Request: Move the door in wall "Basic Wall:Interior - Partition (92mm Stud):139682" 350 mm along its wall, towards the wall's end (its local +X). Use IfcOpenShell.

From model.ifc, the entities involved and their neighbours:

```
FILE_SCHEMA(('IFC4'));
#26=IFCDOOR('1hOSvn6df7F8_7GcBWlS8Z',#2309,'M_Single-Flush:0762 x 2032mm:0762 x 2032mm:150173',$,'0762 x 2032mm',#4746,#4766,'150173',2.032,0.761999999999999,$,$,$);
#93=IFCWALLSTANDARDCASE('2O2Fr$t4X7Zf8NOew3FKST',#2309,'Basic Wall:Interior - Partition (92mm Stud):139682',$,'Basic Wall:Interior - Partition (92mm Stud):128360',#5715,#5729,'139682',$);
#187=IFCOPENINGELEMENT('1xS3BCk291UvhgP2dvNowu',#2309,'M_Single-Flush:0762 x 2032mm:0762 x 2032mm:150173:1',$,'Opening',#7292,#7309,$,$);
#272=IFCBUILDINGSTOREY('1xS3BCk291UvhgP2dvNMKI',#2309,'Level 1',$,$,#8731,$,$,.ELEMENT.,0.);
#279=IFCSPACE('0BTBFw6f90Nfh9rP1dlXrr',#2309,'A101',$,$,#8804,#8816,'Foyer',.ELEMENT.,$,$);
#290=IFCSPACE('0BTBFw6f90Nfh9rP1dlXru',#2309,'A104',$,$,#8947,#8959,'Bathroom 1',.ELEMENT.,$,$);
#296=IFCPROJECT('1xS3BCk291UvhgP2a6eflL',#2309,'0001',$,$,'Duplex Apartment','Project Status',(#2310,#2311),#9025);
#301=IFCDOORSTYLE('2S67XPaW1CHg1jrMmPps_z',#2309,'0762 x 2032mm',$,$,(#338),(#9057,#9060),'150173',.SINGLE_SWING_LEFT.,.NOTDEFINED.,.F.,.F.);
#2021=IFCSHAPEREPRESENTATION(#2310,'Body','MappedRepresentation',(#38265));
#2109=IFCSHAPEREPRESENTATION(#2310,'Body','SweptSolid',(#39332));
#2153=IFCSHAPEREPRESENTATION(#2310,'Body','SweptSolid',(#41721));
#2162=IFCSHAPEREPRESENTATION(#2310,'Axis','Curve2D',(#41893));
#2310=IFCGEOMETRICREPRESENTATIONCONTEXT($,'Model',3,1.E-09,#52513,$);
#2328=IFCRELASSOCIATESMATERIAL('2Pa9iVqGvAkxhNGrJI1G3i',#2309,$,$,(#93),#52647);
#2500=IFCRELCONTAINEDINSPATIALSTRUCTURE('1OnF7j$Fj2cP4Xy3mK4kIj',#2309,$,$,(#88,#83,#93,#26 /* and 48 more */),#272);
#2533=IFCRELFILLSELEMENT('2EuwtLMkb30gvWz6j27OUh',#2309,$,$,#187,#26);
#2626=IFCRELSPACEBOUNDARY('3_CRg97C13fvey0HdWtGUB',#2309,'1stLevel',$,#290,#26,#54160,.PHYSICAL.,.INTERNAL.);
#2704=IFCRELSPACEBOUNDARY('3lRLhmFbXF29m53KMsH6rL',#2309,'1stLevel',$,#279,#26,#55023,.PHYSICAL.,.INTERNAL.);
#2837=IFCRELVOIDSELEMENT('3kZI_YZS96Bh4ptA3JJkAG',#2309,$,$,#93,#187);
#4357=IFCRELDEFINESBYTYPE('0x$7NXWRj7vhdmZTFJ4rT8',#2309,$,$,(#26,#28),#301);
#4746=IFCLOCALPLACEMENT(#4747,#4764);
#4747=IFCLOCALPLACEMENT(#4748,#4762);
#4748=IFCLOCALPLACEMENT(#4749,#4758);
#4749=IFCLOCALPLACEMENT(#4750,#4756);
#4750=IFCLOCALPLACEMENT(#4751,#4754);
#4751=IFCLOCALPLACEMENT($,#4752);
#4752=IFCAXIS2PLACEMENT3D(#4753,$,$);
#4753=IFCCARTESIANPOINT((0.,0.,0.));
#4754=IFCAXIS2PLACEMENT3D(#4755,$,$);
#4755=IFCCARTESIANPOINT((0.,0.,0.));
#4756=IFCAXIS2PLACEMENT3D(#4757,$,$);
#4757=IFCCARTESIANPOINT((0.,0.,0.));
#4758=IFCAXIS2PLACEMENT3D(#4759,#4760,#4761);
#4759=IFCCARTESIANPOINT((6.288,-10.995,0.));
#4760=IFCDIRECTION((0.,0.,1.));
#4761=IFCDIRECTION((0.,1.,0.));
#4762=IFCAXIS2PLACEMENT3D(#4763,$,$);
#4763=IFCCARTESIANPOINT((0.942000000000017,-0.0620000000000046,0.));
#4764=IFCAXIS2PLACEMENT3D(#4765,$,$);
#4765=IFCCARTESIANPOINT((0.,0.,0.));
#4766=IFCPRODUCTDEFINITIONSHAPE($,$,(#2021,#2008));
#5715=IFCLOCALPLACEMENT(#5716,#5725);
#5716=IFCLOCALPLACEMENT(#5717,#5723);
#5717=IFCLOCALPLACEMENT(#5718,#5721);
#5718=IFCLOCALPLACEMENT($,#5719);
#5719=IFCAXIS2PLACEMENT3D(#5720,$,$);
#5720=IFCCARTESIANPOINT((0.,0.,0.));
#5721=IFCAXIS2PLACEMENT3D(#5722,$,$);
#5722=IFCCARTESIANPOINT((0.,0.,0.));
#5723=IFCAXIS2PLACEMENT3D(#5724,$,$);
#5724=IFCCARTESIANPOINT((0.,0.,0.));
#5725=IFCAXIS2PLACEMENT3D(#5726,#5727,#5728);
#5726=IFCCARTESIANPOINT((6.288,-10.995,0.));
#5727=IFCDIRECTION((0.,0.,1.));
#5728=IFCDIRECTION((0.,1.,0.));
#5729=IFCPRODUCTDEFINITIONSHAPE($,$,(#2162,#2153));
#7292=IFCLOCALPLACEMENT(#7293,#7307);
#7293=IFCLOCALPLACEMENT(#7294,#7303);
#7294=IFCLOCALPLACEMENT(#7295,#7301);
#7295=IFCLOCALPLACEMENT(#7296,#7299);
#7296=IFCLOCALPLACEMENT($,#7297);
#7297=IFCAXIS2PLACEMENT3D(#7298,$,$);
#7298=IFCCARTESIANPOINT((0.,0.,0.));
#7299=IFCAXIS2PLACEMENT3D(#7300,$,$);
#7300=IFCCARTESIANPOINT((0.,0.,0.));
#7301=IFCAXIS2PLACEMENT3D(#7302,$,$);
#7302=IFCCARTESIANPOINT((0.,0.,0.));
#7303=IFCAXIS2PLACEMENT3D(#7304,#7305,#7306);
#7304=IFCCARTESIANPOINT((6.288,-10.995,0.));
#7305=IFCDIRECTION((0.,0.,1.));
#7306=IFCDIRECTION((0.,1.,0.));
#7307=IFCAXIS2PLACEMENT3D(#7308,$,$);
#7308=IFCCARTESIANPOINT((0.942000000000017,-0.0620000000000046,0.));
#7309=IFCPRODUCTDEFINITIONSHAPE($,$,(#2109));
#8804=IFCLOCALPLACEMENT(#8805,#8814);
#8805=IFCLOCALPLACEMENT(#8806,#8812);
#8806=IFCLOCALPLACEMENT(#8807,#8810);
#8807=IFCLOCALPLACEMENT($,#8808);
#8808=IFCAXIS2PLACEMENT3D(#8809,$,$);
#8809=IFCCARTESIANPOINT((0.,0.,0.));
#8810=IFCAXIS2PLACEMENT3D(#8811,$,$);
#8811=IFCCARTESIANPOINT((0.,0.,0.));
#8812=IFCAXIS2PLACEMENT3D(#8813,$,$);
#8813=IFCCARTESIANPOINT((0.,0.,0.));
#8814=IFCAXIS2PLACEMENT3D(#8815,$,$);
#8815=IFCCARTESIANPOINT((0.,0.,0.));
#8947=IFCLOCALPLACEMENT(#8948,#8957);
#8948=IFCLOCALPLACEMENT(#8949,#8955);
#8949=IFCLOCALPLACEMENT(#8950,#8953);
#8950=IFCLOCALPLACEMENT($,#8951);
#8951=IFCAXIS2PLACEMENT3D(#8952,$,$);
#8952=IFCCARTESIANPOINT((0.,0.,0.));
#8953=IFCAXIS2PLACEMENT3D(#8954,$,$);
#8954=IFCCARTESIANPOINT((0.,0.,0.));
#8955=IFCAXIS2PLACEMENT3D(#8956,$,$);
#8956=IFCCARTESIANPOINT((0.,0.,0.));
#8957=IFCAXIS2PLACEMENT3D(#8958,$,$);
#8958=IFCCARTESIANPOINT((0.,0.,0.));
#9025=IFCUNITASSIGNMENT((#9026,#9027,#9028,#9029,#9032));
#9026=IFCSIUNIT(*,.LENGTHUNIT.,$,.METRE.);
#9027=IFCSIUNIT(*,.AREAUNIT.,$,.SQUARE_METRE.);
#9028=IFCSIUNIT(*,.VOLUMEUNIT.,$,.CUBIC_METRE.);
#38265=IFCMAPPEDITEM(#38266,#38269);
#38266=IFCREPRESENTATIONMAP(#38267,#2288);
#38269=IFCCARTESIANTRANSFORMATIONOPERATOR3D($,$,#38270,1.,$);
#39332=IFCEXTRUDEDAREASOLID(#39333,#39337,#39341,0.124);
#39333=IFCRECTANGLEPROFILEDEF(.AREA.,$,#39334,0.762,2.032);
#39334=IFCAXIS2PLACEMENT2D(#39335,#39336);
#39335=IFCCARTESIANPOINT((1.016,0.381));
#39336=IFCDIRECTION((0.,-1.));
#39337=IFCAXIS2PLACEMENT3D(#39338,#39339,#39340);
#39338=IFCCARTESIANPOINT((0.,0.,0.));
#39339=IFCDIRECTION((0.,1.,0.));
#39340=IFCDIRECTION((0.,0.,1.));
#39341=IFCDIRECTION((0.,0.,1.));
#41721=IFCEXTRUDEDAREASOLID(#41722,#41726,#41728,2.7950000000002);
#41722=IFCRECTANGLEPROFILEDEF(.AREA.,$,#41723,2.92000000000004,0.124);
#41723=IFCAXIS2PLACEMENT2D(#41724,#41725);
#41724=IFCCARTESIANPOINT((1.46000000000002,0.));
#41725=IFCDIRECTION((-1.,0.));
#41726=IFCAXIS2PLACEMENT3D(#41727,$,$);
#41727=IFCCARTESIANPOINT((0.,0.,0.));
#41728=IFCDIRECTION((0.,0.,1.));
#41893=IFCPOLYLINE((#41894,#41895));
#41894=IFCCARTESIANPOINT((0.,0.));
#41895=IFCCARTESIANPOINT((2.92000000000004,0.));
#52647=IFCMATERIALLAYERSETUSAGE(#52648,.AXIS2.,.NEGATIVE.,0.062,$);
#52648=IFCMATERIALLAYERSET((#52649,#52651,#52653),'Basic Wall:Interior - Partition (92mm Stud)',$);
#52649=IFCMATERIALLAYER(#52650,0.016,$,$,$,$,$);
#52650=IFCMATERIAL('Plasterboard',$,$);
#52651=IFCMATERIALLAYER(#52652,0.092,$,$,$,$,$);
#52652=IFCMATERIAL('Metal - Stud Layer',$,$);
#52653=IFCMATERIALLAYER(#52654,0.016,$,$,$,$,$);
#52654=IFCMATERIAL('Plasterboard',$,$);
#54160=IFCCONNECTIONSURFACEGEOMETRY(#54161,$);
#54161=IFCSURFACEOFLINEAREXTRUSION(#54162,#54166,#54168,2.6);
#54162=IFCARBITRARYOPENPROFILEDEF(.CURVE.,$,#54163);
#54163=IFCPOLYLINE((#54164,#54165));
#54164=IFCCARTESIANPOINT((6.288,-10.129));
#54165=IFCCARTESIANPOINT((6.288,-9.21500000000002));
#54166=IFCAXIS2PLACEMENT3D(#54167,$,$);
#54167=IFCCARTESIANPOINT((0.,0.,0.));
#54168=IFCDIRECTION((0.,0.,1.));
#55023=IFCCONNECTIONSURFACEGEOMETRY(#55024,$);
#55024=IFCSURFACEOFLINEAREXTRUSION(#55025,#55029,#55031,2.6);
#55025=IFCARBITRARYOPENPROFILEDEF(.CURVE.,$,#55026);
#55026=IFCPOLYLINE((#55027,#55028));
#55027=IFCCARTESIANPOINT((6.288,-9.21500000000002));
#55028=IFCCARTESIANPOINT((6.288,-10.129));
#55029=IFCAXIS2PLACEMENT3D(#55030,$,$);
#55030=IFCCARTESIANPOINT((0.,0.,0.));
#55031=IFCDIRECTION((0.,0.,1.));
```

```python
import numpy as np
import ifcopenshell
import ifcopenshell.api.geometry
import ifcopenshell.util.placement

model = ifcopenshell.open("model.ifc")

door = model.by_guid("1hOSvn6df7F8_7GcBWlS8Z")
opening = door.FillsVoids[0].RelatingOpeningElement
wall = opening.VoidsElements[0].RelatingBuildingElement

wall_matrix = ifcopenshell.util.placement.get_local_placement(wall.ObjectPlacement)
shift = wall_matrix[:3, 0] * 0.35
before = ifcopenshell.util.placement.get_local_placement(door.ObjectPlacement)[:3, 3].copy()

# The door is not placed relative to its opening, so move both.
for product in (opening, door):
    matrix = ifcopenshell.util.placement.get_local_placement(product.ObjectPlacement)
    matrix[:3, 3] += shift
    ifcopenshell.api.geometry.edit_object_placement(model, product=product, matrix=matrix, is_si=False)

# Space boundary surfaces are stored in each space's coordinates; move them too.
for rel in door.ProvidesBoundaries:
    if not rel.ConnectionGeometry:
        continue
    surface = rel.ConnectionGeometry.SurfaceOnRelatingElement
    space_matrix = ifcopenshell.util.placement.get_local_placement(rel.RelatingSpace.ObjectPlacement)
    point = np.array(surface.Position.Location.Coordinates) + space_matrix[:3, :3].T @ shift
    surface.Position = model.createIfcAxis2Placement3D(
        model.createIfcCartesianPoint(point.tolist()), surface.Position.Axis, surface.Position.RefDirection
    )

after = ifcopenshell.util.placement.get_local_placement(door.ObjectPlacement)[:3, 3]
print("door moved by", (after - before).round(3) + 0.0)

model.write("model_rev.ifc")
```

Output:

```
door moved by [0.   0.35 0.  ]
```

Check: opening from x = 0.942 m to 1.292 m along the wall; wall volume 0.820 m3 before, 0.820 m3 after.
